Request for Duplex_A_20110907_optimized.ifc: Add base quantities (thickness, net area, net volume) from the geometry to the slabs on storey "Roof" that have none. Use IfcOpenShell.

First a look at what the model holds.

```python
import ifcopenshell
import ifcopenshell.util.element
import ifcopenshell.util.unit

model = ifcopenshell.open("Duplex_A_20110907_optimized.ifc")
print(model.schema)
for unit_type in ("LENGTHUNIT", "AREAUNIT", "VOLUMEUNIT"):
    print(unit_type, ifcopenshell.util.unit.calculate_unit_scale(model, unit_type))
storey = next(s for s in model.by_type("IfcBuildingStorey") if s.Name == "Roof")
slabs = [e for e in ifcopenshell.util.element.get_decomposition(storey) if e.is_a("IfcSlab")]
for e in sorted(slabs, key=lambda e: e.id()):
    print(e.id(), e.is_a(), e.Name, list(ifcopenshell.util.element.get_psets(e, qtos_only=True)), sep=" | ")
```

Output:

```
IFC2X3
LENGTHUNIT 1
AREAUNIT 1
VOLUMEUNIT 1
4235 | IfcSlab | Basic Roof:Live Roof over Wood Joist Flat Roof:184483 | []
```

```python
import ifcopenshell
import ifcopenshell.api.pset
import ifcopenshell.geom
import ifcopenshell.util.element
import ifcopenshell.util.shape
import ifcopenshell.util.unit

model = ifcopenshell.open("Duplex_A_20110907_optimized.ifc")
unit_scale = ifcopenshell.util.unit.calculate_unit_scale(model)
area_scale = ifcopenshell.util.unit.calculate_unit_scale(model, "AREAUNIT")
volume_scale = ifcopenshell.util.unit.calculate_unit_scale(model, "VOLUMEUNIT")
settings = ifcopenshell.geom.settings()

storey = next(s for s in model.by_type("IfcBuildingStorey") if s.Name == "Roof")
slabs = [e for e in ifcopenshell.util.element.get_decomposition(storey) if e.is_a("IfcSlab")]

for e in sorted(slabs, key=lambda e: e.id()):
    if ifcopenshell.util.element.get_psets(e, qtos_only=True, should_inherit=False):
        continue
    # Geometry comes back in metres, in the element's own axes.
    shape = ifcopenshell.geom.create_shape(settings, e)
    values = {
        "Width": ifcopenshell.util.shape.get_z(shape.geometry) / unit_scale,
        "NetArea": ifcopenshell.util.shape.get_footprint_area(shape.geometry) / area_scale,
        "NetVolume": ifcopenshell.util.shape.get_volume(shape.geometry) / volume_scale,
    }
    qto = ifcopenshell.api.pset.add_qto(model, product=e, name="BaseQuantities")
    ifcopenshell.api.pset.edit_qto(model, qto=qto, properties=values)
    print(e.id(), {k: round(v, 3) for k, v in values.items()})

model.write("Duplex_A_20110907_optimized-out.ifc")
```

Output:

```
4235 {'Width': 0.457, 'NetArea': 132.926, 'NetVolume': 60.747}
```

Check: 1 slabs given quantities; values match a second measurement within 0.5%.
